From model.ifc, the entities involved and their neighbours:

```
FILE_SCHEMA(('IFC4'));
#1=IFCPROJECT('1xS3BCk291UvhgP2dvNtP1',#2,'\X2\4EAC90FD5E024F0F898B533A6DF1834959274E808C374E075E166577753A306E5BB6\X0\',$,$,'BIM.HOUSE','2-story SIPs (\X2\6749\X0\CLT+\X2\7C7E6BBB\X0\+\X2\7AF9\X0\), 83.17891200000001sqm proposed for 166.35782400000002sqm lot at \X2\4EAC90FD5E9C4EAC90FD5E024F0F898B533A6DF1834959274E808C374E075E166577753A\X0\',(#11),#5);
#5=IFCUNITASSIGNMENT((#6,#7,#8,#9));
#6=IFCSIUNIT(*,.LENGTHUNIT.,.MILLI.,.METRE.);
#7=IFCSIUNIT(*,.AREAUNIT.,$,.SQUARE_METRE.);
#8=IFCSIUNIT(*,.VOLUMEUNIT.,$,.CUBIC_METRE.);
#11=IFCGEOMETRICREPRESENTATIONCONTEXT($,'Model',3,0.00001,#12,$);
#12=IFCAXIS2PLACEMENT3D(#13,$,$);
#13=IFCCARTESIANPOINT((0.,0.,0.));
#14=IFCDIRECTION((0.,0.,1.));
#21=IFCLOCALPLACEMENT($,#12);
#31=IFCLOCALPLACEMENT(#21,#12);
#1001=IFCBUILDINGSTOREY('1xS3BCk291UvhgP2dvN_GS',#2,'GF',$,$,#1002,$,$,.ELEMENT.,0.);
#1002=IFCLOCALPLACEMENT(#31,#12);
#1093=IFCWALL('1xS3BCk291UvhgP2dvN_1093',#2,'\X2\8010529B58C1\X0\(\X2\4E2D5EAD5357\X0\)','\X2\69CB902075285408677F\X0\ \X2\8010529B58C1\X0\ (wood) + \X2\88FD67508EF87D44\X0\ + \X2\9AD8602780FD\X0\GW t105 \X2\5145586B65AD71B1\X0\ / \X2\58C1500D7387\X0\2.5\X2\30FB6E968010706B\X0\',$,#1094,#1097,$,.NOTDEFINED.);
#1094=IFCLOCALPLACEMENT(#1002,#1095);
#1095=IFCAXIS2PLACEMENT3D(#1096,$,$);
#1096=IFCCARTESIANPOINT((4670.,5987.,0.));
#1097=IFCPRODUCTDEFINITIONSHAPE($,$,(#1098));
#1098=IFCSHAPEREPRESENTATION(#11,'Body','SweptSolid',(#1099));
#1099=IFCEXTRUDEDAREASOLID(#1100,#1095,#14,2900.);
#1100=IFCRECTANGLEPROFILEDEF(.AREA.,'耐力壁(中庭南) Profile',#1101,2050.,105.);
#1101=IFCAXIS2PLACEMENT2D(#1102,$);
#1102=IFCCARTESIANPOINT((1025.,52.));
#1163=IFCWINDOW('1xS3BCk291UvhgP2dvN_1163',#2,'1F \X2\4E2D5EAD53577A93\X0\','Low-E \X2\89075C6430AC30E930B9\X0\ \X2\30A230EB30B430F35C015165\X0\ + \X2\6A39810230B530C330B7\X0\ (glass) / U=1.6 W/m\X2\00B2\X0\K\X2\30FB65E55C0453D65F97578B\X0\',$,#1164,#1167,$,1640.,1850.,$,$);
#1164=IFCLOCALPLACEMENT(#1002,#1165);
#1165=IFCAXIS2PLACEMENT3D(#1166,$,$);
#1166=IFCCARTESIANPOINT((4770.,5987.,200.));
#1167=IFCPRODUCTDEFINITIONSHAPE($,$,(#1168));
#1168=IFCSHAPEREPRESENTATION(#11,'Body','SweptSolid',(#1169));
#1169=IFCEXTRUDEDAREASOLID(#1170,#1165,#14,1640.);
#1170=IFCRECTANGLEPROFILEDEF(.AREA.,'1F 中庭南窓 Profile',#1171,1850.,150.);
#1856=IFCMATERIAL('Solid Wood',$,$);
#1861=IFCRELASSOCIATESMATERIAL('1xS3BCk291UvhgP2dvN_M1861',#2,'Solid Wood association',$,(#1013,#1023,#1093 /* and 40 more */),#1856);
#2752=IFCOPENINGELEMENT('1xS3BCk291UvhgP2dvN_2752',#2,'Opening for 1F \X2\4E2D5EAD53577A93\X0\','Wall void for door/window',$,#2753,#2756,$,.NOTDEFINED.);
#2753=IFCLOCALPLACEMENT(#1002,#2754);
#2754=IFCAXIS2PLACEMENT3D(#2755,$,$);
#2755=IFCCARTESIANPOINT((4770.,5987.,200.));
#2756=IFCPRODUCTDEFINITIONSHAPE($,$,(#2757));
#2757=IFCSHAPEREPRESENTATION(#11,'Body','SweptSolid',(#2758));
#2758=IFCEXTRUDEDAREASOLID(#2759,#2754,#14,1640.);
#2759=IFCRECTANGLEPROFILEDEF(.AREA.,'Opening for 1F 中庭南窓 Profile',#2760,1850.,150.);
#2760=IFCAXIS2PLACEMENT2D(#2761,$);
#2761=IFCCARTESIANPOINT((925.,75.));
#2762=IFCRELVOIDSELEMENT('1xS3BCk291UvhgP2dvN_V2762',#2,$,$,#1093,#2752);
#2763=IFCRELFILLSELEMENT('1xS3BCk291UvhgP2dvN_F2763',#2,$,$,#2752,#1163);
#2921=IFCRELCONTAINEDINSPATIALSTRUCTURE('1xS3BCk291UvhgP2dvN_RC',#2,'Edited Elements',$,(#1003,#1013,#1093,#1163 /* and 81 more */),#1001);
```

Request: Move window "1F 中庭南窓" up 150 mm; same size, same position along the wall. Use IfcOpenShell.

```python
import numpy as np
import ifcopenshell
import ifcopenshell.api.geometry
import ifcopenshell.util.placement
import ifcopenshell.util.unit

model = ifcopenshell.open("model.ifc")
unit_scale = ifcopenshell.util.unit.calculate_unit_scale(model)

window = model.by_id(1163)
opening = window.FillsVoids[0].RelatingOpeningElement
dz = 150.0

shift = np.array([0.0, 0.0, dz])
# The window is not placed relative to its opening, so move both.
for product in (opening, window):
    matrix = ifcopenshell.util.placement.get_local_placement(product.ObjectPlacement)
    matrix[:3, 3] += shift
    ifcopenshell.api.geometry.edit_object_placement(model, product=product, matrix=matrix, is_si=False)

print(f"moved by {dz * unit_scale:+.3f} m")

model.write("model-out.ifc")
```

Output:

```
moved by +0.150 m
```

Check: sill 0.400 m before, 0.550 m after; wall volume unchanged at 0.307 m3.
